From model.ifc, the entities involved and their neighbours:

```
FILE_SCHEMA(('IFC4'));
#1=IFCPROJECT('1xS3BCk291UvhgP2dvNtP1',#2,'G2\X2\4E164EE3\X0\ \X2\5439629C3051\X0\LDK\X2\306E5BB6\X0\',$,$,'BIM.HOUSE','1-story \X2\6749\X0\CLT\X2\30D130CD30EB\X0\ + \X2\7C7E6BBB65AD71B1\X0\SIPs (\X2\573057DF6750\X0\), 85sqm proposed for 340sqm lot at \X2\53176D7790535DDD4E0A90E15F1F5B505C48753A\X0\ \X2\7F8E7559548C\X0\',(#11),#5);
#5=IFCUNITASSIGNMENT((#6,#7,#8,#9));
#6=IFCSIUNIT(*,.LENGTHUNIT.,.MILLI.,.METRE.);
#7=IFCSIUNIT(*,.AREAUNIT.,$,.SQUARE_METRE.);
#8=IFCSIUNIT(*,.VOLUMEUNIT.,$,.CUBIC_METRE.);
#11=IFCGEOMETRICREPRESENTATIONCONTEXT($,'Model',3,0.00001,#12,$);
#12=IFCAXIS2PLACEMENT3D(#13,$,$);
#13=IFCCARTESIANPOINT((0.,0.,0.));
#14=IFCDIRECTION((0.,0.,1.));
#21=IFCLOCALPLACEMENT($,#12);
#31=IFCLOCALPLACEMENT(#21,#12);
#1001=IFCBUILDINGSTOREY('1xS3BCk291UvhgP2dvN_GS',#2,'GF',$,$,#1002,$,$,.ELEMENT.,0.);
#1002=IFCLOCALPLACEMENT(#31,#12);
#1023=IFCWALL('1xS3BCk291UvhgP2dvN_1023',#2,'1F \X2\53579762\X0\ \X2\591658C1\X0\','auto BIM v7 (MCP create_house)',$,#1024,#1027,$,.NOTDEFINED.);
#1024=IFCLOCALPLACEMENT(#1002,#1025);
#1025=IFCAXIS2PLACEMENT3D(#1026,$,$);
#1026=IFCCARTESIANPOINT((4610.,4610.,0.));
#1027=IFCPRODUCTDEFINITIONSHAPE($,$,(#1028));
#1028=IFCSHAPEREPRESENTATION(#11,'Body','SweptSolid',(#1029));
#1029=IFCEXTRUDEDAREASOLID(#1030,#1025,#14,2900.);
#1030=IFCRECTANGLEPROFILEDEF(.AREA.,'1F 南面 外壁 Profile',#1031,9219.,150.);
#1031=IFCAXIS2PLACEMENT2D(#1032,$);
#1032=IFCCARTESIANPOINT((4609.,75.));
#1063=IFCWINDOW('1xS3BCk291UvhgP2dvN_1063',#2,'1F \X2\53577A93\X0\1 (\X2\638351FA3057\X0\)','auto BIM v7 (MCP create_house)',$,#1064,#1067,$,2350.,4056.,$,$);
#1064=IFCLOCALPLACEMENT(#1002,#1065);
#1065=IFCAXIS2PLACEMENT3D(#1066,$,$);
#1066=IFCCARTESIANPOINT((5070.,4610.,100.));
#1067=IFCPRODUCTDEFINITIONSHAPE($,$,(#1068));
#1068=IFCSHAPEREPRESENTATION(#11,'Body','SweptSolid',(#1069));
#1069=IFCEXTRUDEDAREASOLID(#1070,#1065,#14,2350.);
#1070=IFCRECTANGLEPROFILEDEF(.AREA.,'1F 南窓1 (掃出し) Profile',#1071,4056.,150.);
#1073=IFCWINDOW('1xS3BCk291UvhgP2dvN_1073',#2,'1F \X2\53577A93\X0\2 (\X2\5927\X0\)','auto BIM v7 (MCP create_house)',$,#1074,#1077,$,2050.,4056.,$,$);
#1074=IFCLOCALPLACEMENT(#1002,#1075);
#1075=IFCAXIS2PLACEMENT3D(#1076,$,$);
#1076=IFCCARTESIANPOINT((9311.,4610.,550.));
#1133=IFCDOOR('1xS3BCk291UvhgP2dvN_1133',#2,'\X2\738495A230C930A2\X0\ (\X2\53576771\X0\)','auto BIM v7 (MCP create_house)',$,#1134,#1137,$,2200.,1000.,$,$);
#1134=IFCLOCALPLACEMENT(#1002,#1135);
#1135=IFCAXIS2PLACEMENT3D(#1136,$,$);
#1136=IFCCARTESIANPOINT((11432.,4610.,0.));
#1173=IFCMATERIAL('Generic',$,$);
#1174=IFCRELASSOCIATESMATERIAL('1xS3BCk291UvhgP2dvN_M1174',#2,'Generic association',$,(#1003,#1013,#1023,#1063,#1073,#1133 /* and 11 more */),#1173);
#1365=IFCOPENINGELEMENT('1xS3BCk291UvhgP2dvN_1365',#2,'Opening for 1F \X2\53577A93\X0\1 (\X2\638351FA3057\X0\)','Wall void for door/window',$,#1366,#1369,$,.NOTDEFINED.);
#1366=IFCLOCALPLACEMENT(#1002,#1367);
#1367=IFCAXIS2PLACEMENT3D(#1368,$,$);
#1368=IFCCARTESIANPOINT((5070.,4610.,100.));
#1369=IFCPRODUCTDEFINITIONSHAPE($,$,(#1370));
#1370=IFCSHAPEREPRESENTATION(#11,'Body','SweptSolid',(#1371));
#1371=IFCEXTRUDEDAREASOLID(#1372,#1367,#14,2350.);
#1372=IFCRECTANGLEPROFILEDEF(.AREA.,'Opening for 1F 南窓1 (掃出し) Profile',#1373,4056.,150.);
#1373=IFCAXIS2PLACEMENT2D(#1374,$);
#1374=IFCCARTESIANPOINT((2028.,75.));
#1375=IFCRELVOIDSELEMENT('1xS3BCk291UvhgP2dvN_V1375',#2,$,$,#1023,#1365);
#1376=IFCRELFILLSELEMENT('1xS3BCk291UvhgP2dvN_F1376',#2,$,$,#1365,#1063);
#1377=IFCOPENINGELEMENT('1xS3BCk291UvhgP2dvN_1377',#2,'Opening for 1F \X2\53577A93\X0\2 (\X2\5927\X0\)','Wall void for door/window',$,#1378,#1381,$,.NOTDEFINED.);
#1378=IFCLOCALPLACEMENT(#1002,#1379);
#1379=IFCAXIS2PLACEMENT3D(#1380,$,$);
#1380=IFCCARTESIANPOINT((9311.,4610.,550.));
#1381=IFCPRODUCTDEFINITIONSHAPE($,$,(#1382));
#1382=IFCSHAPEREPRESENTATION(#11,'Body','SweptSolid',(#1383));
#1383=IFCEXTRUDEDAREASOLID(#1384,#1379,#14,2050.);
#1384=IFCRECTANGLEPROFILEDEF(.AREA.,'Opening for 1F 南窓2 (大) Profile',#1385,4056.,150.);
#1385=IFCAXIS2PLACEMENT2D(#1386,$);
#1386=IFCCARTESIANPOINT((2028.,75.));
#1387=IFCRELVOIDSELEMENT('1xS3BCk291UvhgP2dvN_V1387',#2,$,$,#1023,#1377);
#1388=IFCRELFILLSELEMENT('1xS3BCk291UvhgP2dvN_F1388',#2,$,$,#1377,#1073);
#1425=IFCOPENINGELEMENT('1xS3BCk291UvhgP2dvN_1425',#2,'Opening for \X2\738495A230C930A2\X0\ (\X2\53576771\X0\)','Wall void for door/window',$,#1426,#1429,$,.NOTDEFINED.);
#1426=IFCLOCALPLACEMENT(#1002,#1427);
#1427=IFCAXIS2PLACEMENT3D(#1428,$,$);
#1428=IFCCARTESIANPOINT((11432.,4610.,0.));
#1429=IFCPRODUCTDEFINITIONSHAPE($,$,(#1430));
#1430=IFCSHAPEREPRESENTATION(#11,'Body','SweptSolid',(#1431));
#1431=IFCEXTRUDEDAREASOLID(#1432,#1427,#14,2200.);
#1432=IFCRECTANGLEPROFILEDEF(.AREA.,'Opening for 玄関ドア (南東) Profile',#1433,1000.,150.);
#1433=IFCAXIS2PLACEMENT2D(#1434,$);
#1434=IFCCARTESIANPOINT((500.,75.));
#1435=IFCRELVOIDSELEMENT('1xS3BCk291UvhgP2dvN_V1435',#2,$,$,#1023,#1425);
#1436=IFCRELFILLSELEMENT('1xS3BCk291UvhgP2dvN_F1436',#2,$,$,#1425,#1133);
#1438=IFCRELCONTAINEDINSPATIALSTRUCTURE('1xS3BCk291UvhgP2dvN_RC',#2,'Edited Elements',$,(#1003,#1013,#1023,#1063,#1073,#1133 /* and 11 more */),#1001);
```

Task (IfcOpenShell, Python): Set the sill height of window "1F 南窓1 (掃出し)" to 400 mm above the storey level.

```python
import numpy as np
import ifcopenshell
import ifcopenshell.api.geometry
import ifcopenshell.geom
import ifcopenshell.util.element
import ifcopenshell.util.placement
import ifcopenshell.util.shape
import ifcopenshell.util.unit

model = ifcopenshell.open("model.ifc")
unit_scale = ifcopenshell.util.unit.calculate_unit_scale(model)

window = model.by_id(1063)
opening = window.FillsVoids[0].RelatingOpeningElement
storey = ifcopenshell.util.element.get_container(window, ifc_class="IfcBuildingStorey")
level = ifcopenshell.util.placement.get_local_placement(storey.ObjectPlacement)[2, 3]

# The opening's origin need not be at the sill, so measure its lowest point.
shape = ifcopenshell.geom.create_shape(ifcopenshell.geom.settings(), opening)
bottom = ifcopenshell.util.shape.get_shape_bottom_elevation(shape, shape.geometry) / unit_scale
dz = level + 0.4 / unit_scale - bottom

shift = np.array([0.0, 0.0, dz])
# The window is not placed relative to its opening, so move both.
for product in (opening, window):
    matrix = ifcopenshell.util.placement.get_local_placement(product.ObjectPlacement)
    matrix[:3, 3] += shift
    ifcopenshell.api.geometry.edit_object_placement(model, product=product, matrix=matrix, is_si=False)

print(f"moved by {dz * unit_scale:+.3f} m")

model.write("model_updated.ifc")
```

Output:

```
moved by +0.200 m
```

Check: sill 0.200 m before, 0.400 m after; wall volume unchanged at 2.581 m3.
